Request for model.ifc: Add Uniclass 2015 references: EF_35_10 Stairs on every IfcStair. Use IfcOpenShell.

First a look at what the model holds.

```python
import ifcopenshell

model = ifcopenshell.open("model.ifc")
print(model.schema)
print("classifications:", [c.Name for c in model.by_type("IfcClassification")])
for ifc_class in ("IfcDoor", "IfcRoof", "IfcStair", "IfcWall", "IfcWindow"):
    print(ifc_class, len(model.by_type(ifc_class)))
```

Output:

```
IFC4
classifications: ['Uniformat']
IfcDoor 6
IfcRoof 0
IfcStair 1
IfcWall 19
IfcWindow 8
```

```python
import ifcopenshell
import ifcopenshell.api.classification

model = ifcopenshell.open("model.ifc")

system = ifcopenshell.api.classification.add_classification(model, classification="Uniclass 2015")

codes = {
    "IfcStair": ("EF_35_10", "Stairs"),
}
for ifc_class, (code, name) in codes.items():
    products = model.by_type(ifc_class)
    ifcopenshell.api.classification.add_reference(
        model, products=products, classification=system, identification=code, name=name
    )
    print(code, len(products))

model.write("model_edited.ifc")
```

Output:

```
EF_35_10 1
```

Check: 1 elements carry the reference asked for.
